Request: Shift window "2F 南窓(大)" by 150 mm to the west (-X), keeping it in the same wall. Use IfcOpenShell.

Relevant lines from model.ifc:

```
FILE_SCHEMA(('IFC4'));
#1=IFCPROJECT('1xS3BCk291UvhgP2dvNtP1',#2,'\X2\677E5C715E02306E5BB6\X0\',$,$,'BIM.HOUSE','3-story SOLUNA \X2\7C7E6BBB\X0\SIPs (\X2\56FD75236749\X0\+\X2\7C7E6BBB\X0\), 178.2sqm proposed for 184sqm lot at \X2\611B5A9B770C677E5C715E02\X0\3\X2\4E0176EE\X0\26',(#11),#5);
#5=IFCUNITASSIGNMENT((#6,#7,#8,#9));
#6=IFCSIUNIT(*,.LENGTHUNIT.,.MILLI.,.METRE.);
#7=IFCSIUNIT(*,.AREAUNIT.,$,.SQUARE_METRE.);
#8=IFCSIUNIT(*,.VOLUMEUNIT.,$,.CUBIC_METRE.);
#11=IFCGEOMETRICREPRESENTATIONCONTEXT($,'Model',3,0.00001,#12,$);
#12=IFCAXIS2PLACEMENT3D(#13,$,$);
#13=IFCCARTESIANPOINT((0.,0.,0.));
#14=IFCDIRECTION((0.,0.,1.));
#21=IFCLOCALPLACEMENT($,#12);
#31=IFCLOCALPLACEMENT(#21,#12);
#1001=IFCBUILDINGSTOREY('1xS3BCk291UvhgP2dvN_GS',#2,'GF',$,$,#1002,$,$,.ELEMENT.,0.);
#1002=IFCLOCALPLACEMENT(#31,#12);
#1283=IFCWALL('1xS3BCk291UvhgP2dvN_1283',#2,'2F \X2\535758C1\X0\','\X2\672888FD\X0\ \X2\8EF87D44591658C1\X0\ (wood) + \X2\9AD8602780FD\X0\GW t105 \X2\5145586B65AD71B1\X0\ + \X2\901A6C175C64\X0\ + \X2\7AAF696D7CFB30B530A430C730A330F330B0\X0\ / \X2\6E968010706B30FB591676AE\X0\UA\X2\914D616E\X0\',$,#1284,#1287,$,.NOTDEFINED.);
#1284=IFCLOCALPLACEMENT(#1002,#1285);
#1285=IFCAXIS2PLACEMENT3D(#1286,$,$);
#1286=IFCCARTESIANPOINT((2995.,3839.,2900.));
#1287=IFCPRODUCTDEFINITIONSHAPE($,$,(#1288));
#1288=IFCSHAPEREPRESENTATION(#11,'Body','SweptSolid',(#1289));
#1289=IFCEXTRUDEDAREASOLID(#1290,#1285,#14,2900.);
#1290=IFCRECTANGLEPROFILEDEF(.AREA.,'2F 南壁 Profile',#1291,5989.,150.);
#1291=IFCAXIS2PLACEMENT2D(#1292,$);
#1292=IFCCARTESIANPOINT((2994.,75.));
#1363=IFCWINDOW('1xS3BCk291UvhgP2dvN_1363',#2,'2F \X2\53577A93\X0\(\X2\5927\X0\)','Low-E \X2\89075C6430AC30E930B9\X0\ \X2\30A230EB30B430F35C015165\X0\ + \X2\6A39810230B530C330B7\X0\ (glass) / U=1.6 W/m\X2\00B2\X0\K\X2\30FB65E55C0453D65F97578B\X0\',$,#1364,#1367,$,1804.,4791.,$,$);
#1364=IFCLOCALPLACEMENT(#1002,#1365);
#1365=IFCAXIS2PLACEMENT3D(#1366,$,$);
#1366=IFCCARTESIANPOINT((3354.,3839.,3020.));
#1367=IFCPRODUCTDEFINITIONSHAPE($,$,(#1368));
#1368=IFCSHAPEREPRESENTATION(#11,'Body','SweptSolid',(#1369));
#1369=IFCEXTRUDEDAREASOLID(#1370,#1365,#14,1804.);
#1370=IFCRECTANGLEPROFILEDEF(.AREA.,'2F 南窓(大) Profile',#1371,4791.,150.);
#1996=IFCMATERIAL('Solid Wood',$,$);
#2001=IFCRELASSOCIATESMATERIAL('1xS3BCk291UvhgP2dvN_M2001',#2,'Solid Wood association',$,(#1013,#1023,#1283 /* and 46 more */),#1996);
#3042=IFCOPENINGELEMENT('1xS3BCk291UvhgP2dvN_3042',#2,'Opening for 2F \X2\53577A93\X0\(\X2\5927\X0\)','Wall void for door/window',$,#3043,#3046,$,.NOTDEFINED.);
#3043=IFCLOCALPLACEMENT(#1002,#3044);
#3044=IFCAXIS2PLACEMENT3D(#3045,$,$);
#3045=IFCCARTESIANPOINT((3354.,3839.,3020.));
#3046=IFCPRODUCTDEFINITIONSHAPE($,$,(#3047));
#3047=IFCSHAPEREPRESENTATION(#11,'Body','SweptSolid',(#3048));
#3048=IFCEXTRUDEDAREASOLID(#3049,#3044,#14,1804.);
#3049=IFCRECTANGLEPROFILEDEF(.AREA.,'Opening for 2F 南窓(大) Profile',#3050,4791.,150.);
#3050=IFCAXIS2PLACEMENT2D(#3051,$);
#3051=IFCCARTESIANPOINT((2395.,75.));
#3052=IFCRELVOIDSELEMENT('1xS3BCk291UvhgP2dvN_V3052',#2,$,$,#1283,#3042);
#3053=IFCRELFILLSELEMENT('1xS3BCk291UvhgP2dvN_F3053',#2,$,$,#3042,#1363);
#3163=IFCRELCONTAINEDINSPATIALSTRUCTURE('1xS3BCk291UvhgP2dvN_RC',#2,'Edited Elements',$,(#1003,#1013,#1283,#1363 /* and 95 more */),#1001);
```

```python
import ifcopenshell
import ifcopenshell.api.geometry
import ifcopenshell.util.placement
import ifcopenshell.util.unit

model = ifcopenshell.open("model.ifc")
unit_scale = ifcopenshell.util.unit.calculate_unit_scale(model)

window = model.by_guid("1xS3BCk291UvhgP2dvN_1363")
opening = window.FillsVoids[0].RelatingOpeningElement
wall = opening.VoidsElements[0].RelatingBuildingElement

wall_matrix = ifcopenshell.util.placement.get_local_placement(wall.ObjectPlacement)
shift = wall_matrix[:3, 0] * -0.15 / unit_scale
before = ifcopenshell.util.placement.get_local_placement(window.ObjectPlacement)[:3, 3].copy()

# The window is not placed relative to its opening, so move both.
for product in (opening, window):
    matrix = ifcopenshell.util.placement.get_local_placement(product.ObjectPlacement)
    matrix[:3, 3] += shift
    ifcopenshell.api.geometry.edit_object_placement(model, product=product, matrix=matrix, is_si=False)

after = ifcopenshell.util.placement.get_local_placement(window.ObjectPlacement)[:3, 3]
print("window moved by", (after - before).round(3) + 0.0)

model.write("model_v2.ifc")
```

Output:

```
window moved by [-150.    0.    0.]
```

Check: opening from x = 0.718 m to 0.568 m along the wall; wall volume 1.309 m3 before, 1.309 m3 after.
